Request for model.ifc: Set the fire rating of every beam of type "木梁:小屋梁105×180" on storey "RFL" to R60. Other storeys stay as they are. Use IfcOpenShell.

First a look at what the model holds.

```python
import ifcopenshell
import ifcopenshell.util.element

model = ifcopenshell.open("model.ifc")
print(model.schema)
storey = next(s for s in model.by_type("IfcBuildingStorey") if s.Name == "RFL")
beams = [e for e in ifcopenshell.util.element.get_decomposition(storey) if e.is_a("IfcBeam")]
seen = {}
for e in beams:
    element_type = ifcopenshell.util.element.get_type(e)
    key = (element_type.Name if element_type != e and element_type else None, ifcopenshell.util.element.get_pset(e, "Pset_BeamCommon", "FireRating"))
    seen[key] = seen.get(key, 0) + 1
for (name, value), count in sorted(seen.items(), key=str):
    print(count, "x", name, "|", value)
```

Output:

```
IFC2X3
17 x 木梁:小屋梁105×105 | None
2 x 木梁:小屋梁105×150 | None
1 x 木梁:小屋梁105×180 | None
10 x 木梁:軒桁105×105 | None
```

```python
import ifcopenshell
import ifcopenshell.api.pset
import ifcopenshell.util.element

model = ifcopenshell.open("model.ifc")

storey = next(s for s in model.by_type("IfcBuildingStorey") if s.Name == "RFL")
beams = [e for e in ifcopenshell.util.element.get_decomposition(storey) if e.is_a("IfcBeam")]

count = 0
for e in beams:
    element_type = ifcopenshell.util.element.get_type(e)
    if element_type in (None, e) or element_type.Name != "木梁:小屋梁105×180":
        continue
    # add_pset returns the element's existing set when there is one.
    pset = ifcopenshell.api.pset.add_pset(model, product=e, name="Pset_BeamCommon")
    ifcopenshell.api.pset.edit_pset(model, pset=pset, properties={"FireRating": "R60"})
    count += 1

print(count, "beams updated")

model.write("model_rev.ifc")
```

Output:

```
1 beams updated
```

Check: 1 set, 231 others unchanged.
